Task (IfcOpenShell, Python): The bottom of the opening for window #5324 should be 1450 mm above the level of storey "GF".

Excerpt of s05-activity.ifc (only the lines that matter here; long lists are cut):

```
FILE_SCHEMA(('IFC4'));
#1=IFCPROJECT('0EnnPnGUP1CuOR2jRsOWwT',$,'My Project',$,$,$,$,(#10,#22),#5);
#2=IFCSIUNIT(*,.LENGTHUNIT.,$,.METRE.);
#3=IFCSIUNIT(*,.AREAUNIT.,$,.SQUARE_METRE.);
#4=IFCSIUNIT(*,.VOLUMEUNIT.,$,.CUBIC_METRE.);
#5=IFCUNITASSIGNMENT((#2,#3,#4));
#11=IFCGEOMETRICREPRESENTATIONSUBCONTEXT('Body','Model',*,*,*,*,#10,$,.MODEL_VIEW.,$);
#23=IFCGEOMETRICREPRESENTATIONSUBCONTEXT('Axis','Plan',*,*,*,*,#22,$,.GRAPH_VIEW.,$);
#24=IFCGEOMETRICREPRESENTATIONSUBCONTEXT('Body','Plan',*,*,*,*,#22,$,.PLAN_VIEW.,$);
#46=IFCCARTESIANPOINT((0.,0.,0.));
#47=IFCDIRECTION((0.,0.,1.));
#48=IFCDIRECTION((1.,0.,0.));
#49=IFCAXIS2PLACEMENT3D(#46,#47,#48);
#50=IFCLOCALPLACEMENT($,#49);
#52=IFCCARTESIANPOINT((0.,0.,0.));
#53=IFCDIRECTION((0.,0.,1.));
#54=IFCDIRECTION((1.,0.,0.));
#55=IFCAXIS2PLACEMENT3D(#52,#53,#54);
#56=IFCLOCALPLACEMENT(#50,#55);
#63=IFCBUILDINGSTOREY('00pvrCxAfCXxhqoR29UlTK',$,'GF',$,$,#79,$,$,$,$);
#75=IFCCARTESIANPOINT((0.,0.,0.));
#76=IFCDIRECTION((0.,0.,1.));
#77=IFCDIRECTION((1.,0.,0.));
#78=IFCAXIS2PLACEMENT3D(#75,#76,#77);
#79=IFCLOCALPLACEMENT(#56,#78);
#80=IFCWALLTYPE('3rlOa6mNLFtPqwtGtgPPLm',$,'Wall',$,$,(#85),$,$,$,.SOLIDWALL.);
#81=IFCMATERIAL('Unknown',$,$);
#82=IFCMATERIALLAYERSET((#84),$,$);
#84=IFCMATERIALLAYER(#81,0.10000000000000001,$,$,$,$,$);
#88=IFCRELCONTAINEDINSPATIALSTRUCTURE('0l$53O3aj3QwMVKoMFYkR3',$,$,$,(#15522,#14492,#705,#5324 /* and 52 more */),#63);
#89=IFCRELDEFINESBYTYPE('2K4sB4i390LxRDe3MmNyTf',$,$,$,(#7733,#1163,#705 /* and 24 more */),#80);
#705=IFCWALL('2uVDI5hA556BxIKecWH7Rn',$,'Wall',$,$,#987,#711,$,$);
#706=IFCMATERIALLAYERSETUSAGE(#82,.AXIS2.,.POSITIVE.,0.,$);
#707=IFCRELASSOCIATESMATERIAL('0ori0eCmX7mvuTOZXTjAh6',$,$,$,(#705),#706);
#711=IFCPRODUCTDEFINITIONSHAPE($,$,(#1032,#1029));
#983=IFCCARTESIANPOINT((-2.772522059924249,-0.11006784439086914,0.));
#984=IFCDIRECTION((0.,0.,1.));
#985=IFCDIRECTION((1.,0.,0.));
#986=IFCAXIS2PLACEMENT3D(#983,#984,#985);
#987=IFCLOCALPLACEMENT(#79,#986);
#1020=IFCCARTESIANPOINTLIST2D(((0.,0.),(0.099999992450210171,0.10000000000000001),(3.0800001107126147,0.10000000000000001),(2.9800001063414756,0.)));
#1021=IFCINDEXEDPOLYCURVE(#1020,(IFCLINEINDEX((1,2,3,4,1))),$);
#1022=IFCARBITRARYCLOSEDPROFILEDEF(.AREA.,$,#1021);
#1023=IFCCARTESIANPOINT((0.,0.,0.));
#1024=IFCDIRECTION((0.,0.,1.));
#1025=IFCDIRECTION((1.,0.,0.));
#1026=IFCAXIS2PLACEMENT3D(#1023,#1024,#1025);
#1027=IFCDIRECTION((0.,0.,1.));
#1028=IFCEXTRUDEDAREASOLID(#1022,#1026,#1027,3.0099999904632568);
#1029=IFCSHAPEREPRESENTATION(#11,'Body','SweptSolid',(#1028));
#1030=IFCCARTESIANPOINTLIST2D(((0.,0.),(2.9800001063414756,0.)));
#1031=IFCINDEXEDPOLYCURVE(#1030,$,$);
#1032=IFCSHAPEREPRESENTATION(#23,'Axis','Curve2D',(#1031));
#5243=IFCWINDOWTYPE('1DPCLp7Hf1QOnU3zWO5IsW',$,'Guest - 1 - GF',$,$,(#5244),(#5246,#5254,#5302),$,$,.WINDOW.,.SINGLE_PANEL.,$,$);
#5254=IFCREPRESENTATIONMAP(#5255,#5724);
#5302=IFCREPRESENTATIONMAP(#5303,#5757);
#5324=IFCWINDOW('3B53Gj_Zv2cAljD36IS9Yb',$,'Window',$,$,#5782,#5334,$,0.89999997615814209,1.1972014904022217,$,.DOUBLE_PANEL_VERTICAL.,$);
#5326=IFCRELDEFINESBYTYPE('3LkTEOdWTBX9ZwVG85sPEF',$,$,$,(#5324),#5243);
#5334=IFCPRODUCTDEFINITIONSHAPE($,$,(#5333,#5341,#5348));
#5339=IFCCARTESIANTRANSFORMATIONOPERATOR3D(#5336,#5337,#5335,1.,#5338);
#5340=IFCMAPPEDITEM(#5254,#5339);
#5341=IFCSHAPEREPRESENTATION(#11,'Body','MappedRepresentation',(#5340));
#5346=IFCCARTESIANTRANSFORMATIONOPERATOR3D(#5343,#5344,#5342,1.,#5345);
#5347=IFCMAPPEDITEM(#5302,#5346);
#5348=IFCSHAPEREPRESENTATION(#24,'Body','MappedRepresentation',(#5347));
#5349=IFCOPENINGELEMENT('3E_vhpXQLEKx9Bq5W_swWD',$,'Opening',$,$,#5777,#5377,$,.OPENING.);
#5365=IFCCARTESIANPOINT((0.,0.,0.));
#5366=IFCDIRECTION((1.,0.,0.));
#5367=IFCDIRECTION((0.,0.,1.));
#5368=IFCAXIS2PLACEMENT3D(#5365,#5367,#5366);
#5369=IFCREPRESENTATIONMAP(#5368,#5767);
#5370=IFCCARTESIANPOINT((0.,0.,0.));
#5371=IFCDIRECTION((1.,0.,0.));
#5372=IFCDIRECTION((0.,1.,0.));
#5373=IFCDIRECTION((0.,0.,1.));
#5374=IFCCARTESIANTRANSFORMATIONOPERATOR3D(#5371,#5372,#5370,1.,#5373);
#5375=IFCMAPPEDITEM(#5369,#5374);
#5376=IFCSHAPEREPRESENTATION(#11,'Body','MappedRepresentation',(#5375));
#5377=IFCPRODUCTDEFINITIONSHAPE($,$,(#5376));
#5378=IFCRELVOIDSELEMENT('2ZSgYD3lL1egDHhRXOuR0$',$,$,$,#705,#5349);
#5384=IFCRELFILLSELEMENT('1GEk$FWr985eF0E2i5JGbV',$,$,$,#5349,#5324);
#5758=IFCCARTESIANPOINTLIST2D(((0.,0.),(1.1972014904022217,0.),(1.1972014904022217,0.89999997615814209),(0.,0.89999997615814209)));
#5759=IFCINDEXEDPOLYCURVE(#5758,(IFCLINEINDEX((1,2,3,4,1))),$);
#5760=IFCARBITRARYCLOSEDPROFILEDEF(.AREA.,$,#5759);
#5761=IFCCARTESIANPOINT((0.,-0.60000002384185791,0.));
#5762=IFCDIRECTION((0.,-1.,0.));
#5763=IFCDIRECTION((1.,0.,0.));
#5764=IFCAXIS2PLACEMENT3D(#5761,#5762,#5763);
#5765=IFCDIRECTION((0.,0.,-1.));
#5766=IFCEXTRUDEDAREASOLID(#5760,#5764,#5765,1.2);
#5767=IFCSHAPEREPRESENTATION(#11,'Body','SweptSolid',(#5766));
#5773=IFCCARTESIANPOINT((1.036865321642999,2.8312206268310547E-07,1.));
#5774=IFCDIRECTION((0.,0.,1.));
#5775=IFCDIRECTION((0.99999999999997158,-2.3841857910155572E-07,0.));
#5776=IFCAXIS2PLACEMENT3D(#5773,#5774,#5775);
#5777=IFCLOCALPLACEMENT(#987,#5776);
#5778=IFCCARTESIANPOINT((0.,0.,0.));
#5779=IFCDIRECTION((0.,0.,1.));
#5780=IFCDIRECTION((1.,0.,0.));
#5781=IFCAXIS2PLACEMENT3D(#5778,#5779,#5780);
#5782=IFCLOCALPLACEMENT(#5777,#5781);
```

```python
import numpy as np
import ifcopenshell
import ifcopenshell.api.geometry
import ifcopenshell.geom
import ifcopenshell.util.element
import ifcopenshell.util.placement
import ifcopenshell.util.shape
import ifcopenshell.util.unit

model = ifcopenshell.open("s05-activity.ifc")
unit_scale = ifcopenshell.util.unit.calculate_unit_scale(model)

window = model.by_id(5324)
opening = window.FillsVoids[0].RelatingOpeningElement
storey = ifcopenshell.util.element.get_container(window, ifc_class="IfcBuildingStorey")
level = ifcopenshell.util.placement.get_local_placement(storey.ObjectPlacement)[2, 3]

# The opening's origin need not be at the sill, so measure its lowest point.
shape = ifcopenshell.geom.create_shape(ifcopenshell.geom.settings(), opening)
bottom = ifcopenshell.util.shape.get_shape_bottom_elevation(shape, shape.geometry) / unit_scale
dz = level + 1.45 / unit_scale - bottom

shift = np.array([0.0, 0.0, dz])
# The window is placed relative to its opening, so it follows when the opening moves.
matrix = ifcopenshell.util.placement.get_local_placement(opening.ObjectPlacement)
matrix[:3, 3] += shift
ifcopenshell.api.geometry.edit_object_placement(
    model, product=opening, matrix=matrix, is_si=False, should_transform_children=True
)

print(f"moved by {dz * unit_scale:+.3f} m")

model.write("s05-activity_edited.ifc")
```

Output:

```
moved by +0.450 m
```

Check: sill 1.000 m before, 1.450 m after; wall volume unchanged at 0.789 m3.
